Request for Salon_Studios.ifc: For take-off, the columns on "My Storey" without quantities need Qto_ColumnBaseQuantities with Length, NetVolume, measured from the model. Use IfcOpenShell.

First a look at what the model holds.

```python
import ifcopenshell
import ifcopenshell.util.element
import ifcopenshell.util.unit

model = ifcopenshell.open("Salon_Studios.ifc")
print(model.schema)
for unit_type in ("LENGTHUNIT", "AREAUNIT", "VOLUMEUNIT"):
    print(unit_type, ifcopenshell.util.unit.calculate_unit_scale(model, unit_type))
storey = next(s for s in model.by_type("IfcBuildingStorey") if s.Name == "My Storey")
columns = [e for e in ifcopenshell.util.element.get_decomposition(storey) if e.is_a("IfcColumn")]
for e in sorted(columns, key=lambda e: e.id()):
    print(e.id(), e.is_a(), e.Name, list(ifcopenshell.util.element.get_psets(e, qtos_only=True)), sep=" | ")
```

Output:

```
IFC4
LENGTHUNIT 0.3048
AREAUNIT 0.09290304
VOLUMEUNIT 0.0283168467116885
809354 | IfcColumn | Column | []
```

```python
import ifcopenshell
import ifcopenshell.api.pset
import ifcopenshell.geom
import ifcopenshell.util.element
import ifcopenshell.util.shape
import ifcopenshell.util.unit

model = ifcopenshell.open("Salon_Studios.ifc")
unit_scale = ifcopenshell.util.unit.calculate_unit_scale(model)
volume_scale = ifcopenshell.util.unit.calculate_unit_scale(model, "VOLUMEUNIT")
settings = ifcopenshell.geom.settings()

storey = next(s for s in model.by_type("IfcBuildingStorey") if s.Name == "My Storey")
columns = [e for e in ifcopenshell.util.element.get_decomposition(storey) if e.is_a("IfcColumn")]

for e in sorted(columns, key=lambda e: e.id()):
    if ifcopenshell.util.element.get_psets(e, qtos_only=True, should_inherit=False):
        continue
    # Geometry comes back in metres, in the element's own axes.
    shape = ifcopenshell.geom.create_shape(settings, e)
    values = {
        "Length": ifcopenshell.util.shape.get_z(shape.geometry) / unit_scale,
        "NetVolume": ifcopenshell.util.shape.get_volume(shape.geometry) / volume_scale,
    }
    qto = ifcopenshell.api.pset.add_qto(model, product=e, name="Qto_ColumnBaseQuantities")
    ifcopenshell.api.pset.edit_qto(model, qto=qto, properties=values)
    print(e.id(), {k: round(v, 3) for k, v in values.items()})

model.write("Salon_Studios_updated.ifc")
```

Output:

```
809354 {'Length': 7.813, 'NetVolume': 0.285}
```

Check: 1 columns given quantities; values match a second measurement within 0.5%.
